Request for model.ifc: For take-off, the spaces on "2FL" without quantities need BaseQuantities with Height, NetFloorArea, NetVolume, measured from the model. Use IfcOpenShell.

First a look at what the model holds.

```python
import ifcopenshell
import ifcopenshell.util.element
import ifcopenshell.util.unit

model = ifcopenshell.open("model.ifc")
print(model.schema)
for unit_type in ("LENGTHUNIT", "AREAUNIT", "VOLUMEUNIT"):
    print(unit_type, ifcopenshell.util.unit.calculate_unit_scale(model, unit_type))
storey = next(s for s in model.by_type("IfcBuildingStorey") if s.Name == "2FL")
spaces = [e for e in ifcopenshell.util.element.get_decomposition(storey) if e.is_a("IfcSpace")]
for e in sorted(spaces, key=lambda e: e.id()):
    print(e.id(), e.is_a(), e.Name, list(ifcopenshell.util.element.get_psets(e, qtos_only=True)), sep=" | ")
```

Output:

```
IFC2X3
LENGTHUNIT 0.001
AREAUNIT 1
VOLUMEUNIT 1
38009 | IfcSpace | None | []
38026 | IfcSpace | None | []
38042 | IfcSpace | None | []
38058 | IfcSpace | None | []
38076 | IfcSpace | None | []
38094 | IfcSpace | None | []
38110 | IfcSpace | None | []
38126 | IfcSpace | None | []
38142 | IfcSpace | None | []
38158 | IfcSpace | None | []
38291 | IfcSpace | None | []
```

```python
import ifcopenshell
import ifcopenshell.api.pset
import ifcopenshell.geom
import ifcopenshell.util.element
import ifcopenshell.util.shape
import ifcopenshell.util.unit

model = ifcopenshell.open("model.ifc")
unit_scale = ifcopenshell.util.unit.calculate_unit_scale(model)
area_scale = ifcopenshell.util.unit.calculate_unit_scale(model, "AREAUNIT")
volume_scale = ifcopenshell.util.unit.calculate_unit_scale(model, "VOLUMEUNIT")
settings = ifcopenshell.geom.settings()

storey = next(s for s in model.by_type("IfcBuildingStorey") if s.Name == "2FL")
spaces = [e for e in ifcopenshell.util.element.get_decomposition(storey) if e.is_a("IfcSpace")]

for e in sorted(spaces, key=lambda e: e.id()):
    if ifcopenshell.util.element.get_psets(e, qtos_only=True, should_inherit=False):
        continue
    # Geometry comes back in metres, in the element's own axes.
    shape = ifcopenshell.geom.create_shape(settings, e)
    values = {
        "Height": ifcopenshell.util.shape.get_z(shape.geometry) / unit_scale,
        "NetFloorArea": ifcopenshell.util.shape.get_footprint_area(shape.geometry) / area_scale,
        "NetVolume": ifcopenshell.util.shape.get_volume(shape.geometry) / volume_scale,
    }
    qto = ifcopenshell.api.pset.add_qto(model, product=e, name="BaseQuantities")
    ifcopenshell.api.pset.edit_qto(model, qto=qto, properties=values)
    print(e.id(), {k: round(v, 3) for k, v in values.items()})

model.write("model_updated.ifc")
```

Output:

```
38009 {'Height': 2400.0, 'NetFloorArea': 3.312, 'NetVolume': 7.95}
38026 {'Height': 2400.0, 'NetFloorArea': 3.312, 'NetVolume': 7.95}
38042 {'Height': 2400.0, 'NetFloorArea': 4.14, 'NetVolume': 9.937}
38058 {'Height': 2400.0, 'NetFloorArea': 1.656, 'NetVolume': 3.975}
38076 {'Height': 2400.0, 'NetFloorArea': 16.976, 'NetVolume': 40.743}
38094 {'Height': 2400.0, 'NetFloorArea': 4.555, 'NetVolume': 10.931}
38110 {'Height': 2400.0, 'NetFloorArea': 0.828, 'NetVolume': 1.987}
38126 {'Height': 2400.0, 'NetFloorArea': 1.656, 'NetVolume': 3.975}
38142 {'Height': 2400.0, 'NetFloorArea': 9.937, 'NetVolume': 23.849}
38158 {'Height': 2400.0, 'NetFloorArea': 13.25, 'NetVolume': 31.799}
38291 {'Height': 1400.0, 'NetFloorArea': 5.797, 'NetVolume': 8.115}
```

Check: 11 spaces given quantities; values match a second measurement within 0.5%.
